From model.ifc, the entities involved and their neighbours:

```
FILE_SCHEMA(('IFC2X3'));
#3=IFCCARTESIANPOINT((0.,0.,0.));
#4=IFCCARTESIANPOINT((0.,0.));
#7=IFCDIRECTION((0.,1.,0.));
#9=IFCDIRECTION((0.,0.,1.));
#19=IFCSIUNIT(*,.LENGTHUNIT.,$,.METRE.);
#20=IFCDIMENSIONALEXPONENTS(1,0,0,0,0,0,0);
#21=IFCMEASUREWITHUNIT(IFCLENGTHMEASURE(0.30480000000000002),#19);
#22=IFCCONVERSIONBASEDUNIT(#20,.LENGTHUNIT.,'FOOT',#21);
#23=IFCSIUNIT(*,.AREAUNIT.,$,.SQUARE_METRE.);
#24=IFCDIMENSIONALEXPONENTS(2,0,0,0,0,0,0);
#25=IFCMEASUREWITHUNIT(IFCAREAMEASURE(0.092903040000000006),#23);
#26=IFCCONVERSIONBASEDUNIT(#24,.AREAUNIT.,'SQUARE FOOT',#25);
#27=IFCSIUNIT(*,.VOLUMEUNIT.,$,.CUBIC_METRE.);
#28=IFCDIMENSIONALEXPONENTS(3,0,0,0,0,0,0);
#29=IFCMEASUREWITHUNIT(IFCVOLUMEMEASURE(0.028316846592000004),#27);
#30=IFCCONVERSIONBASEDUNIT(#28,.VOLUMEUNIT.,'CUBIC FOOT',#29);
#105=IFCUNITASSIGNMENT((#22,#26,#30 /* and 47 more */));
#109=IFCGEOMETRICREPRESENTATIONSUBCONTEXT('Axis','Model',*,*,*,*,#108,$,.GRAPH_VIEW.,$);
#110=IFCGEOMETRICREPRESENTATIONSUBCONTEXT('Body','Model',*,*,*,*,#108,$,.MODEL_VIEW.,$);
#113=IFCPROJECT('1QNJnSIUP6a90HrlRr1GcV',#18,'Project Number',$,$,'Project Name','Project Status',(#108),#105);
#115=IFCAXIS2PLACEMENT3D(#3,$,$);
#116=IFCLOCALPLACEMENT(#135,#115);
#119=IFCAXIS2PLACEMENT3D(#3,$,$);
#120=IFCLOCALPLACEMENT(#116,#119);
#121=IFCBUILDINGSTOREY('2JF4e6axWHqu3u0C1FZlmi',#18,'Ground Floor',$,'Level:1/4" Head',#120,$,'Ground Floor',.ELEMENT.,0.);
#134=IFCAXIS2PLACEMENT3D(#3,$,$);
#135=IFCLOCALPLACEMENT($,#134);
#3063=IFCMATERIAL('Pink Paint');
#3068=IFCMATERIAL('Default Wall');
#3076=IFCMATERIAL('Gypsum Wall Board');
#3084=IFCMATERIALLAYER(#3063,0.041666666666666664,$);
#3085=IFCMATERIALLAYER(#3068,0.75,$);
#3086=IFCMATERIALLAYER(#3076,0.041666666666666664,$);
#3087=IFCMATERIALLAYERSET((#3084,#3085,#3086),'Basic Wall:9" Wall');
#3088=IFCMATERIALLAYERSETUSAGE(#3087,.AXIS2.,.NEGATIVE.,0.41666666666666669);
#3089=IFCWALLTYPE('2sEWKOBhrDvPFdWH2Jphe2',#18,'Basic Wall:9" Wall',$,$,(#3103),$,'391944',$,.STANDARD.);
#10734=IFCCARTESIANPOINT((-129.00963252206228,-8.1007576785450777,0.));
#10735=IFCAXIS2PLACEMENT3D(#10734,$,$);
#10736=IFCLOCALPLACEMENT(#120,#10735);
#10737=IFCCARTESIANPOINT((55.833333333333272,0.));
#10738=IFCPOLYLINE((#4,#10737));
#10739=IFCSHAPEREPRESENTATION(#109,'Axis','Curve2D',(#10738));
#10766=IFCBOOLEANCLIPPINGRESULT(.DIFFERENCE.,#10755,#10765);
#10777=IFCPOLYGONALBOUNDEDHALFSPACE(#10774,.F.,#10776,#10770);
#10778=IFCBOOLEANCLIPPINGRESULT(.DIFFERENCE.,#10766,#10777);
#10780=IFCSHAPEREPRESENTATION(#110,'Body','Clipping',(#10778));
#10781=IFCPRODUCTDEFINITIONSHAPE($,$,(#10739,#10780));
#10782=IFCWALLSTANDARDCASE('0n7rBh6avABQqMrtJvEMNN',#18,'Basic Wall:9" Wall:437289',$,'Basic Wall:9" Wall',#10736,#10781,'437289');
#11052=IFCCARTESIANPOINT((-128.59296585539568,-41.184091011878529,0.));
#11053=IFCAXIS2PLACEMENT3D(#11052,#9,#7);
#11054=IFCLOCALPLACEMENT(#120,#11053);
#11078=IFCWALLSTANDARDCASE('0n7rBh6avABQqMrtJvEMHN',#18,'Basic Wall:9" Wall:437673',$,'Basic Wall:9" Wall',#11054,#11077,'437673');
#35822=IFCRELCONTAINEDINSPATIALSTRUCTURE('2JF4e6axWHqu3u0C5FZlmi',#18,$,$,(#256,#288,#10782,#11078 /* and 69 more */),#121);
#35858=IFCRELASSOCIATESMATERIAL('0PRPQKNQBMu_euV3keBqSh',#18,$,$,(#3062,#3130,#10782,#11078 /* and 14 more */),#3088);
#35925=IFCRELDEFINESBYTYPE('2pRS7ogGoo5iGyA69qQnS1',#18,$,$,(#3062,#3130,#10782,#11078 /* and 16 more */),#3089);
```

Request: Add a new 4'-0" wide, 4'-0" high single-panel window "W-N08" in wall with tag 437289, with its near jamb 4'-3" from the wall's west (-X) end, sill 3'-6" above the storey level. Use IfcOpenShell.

```python
import numpy as np
import ifcopenshell
import ifcopenshell.api.feature
import ifcopenshell.api.geometry
import ifcopenshell.api.root
import ifcopenshell.api.spatial
import ifcopenshell.api.type
import ifcopenshell.geom
import ifcopenshell.util.element
import ifcopenshell.util.placement
import ifcopenshell.util.representation
import ifcopenshell.util.shape
import ifcopenshell.util.unit

model = ifcopenshell.open("model.ifc")
unit_scale = ifcopenshell.util.unit.calculate_unit_scale(model)
settings = ifcopenshell.geom.settings()


def volume(element):
    """Net volume in cubic metres, openings subtracted."""
    shape = ifcopenshell.geom.create_shape(settings, element)
    return ifcopenshell.util.shape.get_volume(shape.geometry)


wall = model.by_guid("0n7rBh6avABQqMrtJvEMNN")
storey = ifcopenshell.util.element.get_container(wall, ifc_class="IfcBuildingStorey")
context = ifcopenshell.util.representation.get_context(model, "Model", "Body", "MODEL_VIEW")
before = volume(wall)

width, height, from_end, sill = 1.2192, 1.2192, 1.2954, 1.0668  # metres

# The wall runs along its own X axis, and the end named is its -X end.
wall_shape = ifcopenshell.geom.create_shape(settings, wall)
x, y, z = ifcopenshell.util.shape.get_vertices(wall_shape.geometry).T
start = x.min() + from_end
face, thickness = float(y.min()), float(y.max() - y.min())
wall_matrix = ifcopenshell.util.placement.get_local_placement(wall.ObjectPlacement)
level = ifcopenshell.util.placement.get_local_placement(storey.ObjectPlacement)[2, 3]


def in_wall(x, y):
    """Placement at x, y metres in the wall's axes, at sill height."""
    matrix = wall_matrix.copy()
    matrix[:, 3] = wall_matrix @ np.array([x / unit_scale, y / unit_scale, 0.0, 1.0])
    matrix[2, 3] = level + sill / unit_scale
    return matrix


# Opening: a box that overshoots both wall faces by 50 mm.
opening = ifcopenshell.api.root.create_entity(model, ifc_class="IfcOpeningElement")
box = ifcopenshell.api.geometry.add_wall_representation(
    model, context=context, length=width, height=height, thickness=thickness + 0.1
)
ifcopenshell.api.geometry.assign_representation(model, product=opening, representation=box)
ifcopenshell.api.geometry.edit_object_placement(model, product=opening, matrix=in_wall(start, face - 0.05), is_si=False)
ifcopenshell.api.feature.add_feature(model, feature=opening, element=wall)

window = ifcopenshell.api.root.create_entity(model, ifc_class="IfcWindow", name="W-N08")
window.OverallWidth, window.OverallHeight = width / unit_scale, height / unit_scale
body = ifcopenshell.api.geometry.add_window_representation(
    model,
    context=context,
    overall_width=window.OverallWidth,
    overall_height=window.OverallHeight,
    partition_type="SINGLE_PANEL",
)
ifcopenshell.api.geometry.assign_representation(model, product=window, representation=body)
ifcopenshell.api.spatial.assign_container(model, products=[window], relating_structure=storey)
fills = ifcopenshell.api.feature.add_filling(model, opening=opening, element=window)
fills.OwnerHistory = window.OwnerHistory  # required in IFC2X3

# IFC2X3 keeps the operation on the window style.
style = ifcopenshell.api.root.create_entity(model, ifc_class="IfcWindowStyle", name="W-N08")
style.OperationType, style.ConstructionType = "SINGLE_PANEL", "NOTDEFINED"
style.ParameterTakesPrecedence = style.Sizeable = False
ifcopenshell.api.type.assign_type(model, related_objects=[window], relating_type=style)

# Centre the window in the wall's thickness.
ifcopenshell.api.geometry.edit_object_placement(model, product=window, matrix=in_wall(start, face), is_si=False)
window_shape = ifcopenshell.geom.create_shape(settings, window)
depth = ifcopenshell.util.shape.get_vertices(window_shape.geometry)[:, 1]
offset = face + thickness / 2 - (depth.min() + depth.max()) / 2
ifcopenshell.api.geometry.edit_object_placement(model, product=window, matrix=in_wall(start, offset), is_si=False)

after = volume(wall)

print(f"wall volume {before:.3f} -> {after:.3f} m3")

model.write("model_rev.ifc")
```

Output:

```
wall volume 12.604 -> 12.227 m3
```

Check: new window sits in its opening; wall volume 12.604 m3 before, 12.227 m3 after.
